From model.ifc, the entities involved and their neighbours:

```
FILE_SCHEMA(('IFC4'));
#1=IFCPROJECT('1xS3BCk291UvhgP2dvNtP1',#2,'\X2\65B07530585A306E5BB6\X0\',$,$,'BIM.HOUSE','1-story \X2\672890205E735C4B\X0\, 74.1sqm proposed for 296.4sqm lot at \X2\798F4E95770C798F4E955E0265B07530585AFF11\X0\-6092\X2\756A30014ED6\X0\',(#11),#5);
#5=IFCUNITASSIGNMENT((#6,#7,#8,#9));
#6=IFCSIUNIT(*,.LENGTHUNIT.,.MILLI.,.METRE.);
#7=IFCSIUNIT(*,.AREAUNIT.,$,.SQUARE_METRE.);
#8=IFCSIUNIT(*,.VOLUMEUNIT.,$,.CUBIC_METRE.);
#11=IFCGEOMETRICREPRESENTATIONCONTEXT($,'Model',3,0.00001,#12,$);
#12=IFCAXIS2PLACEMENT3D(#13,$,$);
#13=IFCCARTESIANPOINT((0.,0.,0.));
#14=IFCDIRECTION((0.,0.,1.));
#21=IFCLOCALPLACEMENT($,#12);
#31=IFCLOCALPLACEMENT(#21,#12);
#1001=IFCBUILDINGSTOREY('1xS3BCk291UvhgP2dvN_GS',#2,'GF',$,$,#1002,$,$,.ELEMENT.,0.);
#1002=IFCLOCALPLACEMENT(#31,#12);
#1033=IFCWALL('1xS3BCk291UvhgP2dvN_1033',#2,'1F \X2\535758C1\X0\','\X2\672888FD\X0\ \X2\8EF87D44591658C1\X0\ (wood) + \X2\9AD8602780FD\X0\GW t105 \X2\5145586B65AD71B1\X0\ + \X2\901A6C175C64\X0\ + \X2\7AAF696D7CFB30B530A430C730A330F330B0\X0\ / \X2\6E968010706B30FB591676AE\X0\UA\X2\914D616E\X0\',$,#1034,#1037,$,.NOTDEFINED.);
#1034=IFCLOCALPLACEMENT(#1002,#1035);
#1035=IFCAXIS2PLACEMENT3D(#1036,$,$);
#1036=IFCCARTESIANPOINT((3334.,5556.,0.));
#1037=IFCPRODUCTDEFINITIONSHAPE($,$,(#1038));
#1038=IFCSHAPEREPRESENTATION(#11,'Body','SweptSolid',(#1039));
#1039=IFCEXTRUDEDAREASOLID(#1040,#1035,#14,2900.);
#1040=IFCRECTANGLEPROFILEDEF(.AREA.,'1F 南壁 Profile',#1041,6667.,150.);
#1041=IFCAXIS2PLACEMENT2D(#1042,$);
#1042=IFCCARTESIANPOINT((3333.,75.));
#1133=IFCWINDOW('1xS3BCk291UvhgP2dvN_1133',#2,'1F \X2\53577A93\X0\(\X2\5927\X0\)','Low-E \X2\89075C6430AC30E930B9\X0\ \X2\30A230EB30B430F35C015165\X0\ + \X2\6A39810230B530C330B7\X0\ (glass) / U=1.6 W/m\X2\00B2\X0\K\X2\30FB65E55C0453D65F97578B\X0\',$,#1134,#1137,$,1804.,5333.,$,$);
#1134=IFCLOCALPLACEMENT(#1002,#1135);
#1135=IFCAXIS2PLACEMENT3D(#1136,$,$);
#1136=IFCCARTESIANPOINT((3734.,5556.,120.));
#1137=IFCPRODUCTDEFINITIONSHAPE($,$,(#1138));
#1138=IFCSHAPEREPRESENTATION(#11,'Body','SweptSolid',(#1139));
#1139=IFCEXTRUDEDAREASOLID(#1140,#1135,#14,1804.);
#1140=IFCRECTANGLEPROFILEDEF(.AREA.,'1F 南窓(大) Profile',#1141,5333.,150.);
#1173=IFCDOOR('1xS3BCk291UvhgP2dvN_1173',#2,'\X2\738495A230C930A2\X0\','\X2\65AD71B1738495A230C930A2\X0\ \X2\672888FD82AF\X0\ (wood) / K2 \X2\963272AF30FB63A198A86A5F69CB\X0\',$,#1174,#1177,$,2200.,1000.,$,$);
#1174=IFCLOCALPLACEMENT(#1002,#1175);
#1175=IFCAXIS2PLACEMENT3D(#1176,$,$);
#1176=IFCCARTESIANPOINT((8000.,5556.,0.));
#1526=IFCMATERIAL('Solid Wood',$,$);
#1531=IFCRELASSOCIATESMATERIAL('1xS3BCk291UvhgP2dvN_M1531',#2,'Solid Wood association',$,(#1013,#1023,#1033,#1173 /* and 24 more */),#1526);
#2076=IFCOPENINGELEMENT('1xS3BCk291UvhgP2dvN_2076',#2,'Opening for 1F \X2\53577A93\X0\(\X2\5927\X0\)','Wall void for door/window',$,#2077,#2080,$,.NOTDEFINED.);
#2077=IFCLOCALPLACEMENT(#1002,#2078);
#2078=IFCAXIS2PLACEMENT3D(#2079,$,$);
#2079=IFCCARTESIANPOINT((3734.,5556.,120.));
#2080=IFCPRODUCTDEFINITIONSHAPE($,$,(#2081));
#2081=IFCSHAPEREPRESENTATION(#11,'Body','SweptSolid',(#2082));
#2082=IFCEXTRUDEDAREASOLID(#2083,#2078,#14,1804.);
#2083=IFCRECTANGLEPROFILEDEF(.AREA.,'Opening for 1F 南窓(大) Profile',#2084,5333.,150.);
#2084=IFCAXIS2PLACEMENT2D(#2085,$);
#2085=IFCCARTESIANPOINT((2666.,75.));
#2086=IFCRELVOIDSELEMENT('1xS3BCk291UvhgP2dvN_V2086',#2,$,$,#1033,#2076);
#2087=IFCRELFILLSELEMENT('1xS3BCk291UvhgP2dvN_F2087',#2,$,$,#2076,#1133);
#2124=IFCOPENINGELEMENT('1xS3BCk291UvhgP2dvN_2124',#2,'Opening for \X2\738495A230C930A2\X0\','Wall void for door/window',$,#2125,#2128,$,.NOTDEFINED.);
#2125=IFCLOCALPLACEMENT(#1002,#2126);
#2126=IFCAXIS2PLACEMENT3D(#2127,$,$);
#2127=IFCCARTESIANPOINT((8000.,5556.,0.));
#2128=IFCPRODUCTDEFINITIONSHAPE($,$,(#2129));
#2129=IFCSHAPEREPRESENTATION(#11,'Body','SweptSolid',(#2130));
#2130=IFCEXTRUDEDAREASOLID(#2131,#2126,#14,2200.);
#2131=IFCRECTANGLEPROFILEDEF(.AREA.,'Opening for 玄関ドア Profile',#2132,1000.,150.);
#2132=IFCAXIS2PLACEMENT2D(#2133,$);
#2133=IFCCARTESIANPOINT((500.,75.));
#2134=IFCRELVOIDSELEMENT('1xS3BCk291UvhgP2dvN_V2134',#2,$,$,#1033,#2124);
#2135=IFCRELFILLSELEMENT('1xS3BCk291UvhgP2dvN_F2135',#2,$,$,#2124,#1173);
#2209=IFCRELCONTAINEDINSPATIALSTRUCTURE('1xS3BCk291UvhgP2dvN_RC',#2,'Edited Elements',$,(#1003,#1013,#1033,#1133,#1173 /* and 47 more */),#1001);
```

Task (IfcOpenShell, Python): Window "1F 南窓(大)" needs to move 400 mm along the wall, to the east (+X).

```python
import ifcopenshell
import ifcopenshell.api.geometry
import ifcopenshell.util.placement
import ifcopenshell.util.unit

model = ifcopenshell.open("model.ifc")
unit_scale = ifcopenshell.util.unit.calculate_unit_scale(model)

window = model.by_id(1133)
opening = window.FillsVoids[0].RelatingOpeningElement
wall = opening.VoidsElements[0].RelatingBuildingElement

wall_matrix = ifcopenshell.util.placement.get_local_placement(wall.ObjectPlacement)
shift = wall_matrix[:3, 0] * 0.4 / unit_scale
before = ifcopenshell.util.placement.get_local_placement(window.ObjectPlacement)[:3, 3].copy()

# The window is not placed relative to its opening, so move both.
for product in (opening, window):
    matrix = ifcopenshell.util.placement.get_local_placement(product.ObjectPlacement)
    matrix[:3, 3] += shift
    ifcopenshell.api.geometry.edit_object_placement(model, product=product, matrix=matrix, is_si=False)

after = ifcopenshell.util.placement.get_local_placement(window.ObjectPlacement)[:3, 3]
print("window moved by", (after - before).round(3) + 0.0)

model.write("model-out.ifc")
```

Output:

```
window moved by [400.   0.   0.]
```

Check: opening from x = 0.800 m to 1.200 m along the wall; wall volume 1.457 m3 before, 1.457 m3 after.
